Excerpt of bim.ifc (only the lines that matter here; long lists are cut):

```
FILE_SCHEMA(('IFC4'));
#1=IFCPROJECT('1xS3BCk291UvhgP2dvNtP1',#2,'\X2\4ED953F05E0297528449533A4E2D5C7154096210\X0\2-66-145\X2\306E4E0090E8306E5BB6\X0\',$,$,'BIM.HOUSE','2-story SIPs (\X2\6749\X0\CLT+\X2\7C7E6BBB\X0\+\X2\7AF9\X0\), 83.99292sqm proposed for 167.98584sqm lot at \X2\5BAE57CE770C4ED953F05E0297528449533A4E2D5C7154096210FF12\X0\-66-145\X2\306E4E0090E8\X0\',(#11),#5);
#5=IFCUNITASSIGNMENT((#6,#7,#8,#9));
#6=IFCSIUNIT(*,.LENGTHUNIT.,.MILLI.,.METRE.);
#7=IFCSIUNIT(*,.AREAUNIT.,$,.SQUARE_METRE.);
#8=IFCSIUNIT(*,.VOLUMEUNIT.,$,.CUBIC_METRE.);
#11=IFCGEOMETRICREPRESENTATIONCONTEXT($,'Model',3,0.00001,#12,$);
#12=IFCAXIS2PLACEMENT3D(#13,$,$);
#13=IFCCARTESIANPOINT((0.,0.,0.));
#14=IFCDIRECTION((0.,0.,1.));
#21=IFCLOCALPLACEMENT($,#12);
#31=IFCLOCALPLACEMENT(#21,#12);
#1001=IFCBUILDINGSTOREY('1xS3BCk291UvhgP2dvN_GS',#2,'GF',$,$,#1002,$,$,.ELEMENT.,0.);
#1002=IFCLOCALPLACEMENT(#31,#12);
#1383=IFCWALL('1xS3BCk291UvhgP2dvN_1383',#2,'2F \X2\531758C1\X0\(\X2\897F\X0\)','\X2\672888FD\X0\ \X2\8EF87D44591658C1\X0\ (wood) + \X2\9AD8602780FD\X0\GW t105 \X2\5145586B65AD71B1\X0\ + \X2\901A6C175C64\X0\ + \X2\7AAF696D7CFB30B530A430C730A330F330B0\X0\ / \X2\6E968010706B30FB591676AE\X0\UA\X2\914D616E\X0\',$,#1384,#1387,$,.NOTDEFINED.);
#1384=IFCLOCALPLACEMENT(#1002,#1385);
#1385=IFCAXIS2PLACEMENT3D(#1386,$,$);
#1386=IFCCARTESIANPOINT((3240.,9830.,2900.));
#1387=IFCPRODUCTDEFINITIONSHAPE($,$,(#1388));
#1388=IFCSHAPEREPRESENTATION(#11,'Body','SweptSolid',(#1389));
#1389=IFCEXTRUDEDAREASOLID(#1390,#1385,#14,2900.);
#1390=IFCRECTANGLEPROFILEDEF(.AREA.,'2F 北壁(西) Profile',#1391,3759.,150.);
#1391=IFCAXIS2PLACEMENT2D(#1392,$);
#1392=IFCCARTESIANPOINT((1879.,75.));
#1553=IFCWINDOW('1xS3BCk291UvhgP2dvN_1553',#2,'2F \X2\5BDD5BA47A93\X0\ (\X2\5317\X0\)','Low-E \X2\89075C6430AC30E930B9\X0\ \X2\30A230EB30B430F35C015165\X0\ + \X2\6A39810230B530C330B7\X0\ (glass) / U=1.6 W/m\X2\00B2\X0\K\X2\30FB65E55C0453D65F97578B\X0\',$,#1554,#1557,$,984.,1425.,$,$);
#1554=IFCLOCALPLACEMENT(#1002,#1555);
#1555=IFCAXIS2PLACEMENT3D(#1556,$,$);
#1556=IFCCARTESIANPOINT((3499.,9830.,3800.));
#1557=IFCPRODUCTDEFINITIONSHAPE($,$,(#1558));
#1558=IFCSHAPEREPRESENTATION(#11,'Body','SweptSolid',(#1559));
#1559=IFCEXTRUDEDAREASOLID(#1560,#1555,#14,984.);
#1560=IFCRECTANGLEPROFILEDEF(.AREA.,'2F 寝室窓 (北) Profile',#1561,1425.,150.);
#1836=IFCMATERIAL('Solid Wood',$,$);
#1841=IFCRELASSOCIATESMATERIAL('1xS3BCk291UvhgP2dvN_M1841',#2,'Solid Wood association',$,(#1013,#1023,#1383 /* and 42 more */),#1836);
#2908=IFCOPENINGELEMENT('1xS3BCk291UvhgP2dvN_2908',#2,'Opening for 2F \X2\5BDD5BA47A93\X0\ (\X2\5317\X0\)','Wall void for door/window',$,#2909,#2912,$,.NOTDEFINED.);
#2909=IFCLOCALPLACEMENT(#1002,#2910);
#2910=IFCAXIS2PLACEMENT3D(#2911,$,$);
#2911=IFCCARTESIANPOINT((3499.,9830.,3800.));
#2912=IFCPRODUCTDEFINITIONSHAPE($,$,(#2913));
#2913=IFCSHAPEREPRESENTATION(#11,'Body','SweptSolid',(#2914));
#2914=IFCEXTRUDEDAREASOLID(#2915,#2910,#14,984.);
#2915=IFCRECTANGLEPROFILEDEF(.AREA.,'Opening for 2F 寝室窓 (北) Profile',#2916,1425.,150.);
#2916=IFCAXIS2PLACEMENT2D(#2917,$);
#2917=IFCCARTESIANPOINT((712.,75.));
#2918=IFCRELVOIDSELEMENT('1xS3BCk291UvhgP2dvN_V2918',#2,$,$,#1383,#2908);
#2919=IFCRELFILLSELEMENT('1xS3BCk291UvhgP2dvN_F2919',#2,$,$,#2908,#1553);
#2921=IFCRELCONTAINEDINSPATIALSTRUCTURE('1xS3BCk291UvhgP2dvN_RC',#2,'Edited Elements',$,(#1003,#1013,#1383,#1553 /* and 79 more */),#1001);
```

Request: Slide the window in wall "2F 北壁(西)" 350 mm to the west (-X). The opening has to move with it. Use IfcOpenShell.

```python
import ifcopenshell
import ifcopenshell.api.geometry
import ifcopenshell.util.placement

model = ifcopenshell.open("bim.ifc")

window = model.by_guid("1xS3BCk291UvhgP2dvN_1553")
opening = window.FillsVoids[0].RelatingOpeningElement
wall = opening.VoidsElements[0].RelatingBuildingElement

wall_matrix = ifcopenshell.util.placement.get_local_placement(wall.ObjectPlacement)
shift = wall_matrix[:3, 0] * -350.0
before = ifcopenshell.util.placement.get_local_placement(window.ObjectPlacement)[:3, 3].copy()

# The window is not placed relative to its opening, so move both.
for product in (opening, window):
    matrix = ifcopenshell.util.placement.get_local_placement(product.ObjectPlacement)
    matrix[:3, 3] += shift
    ifcopenshell.api.geometry.edit_object_placement(model, product=product, matrix=matrix, is_si=False)

after = ifcopenshell.util.placement.get_local_placement(window.ObjectPlacement)[:3, 3]
print("window moved by", (after - before).round(3) + 0.0)

model.write("bim_rev.ifc")
```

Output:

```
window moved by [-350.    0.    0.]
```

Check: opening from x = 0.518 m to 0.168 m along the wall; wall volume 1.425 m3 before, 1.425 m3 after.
